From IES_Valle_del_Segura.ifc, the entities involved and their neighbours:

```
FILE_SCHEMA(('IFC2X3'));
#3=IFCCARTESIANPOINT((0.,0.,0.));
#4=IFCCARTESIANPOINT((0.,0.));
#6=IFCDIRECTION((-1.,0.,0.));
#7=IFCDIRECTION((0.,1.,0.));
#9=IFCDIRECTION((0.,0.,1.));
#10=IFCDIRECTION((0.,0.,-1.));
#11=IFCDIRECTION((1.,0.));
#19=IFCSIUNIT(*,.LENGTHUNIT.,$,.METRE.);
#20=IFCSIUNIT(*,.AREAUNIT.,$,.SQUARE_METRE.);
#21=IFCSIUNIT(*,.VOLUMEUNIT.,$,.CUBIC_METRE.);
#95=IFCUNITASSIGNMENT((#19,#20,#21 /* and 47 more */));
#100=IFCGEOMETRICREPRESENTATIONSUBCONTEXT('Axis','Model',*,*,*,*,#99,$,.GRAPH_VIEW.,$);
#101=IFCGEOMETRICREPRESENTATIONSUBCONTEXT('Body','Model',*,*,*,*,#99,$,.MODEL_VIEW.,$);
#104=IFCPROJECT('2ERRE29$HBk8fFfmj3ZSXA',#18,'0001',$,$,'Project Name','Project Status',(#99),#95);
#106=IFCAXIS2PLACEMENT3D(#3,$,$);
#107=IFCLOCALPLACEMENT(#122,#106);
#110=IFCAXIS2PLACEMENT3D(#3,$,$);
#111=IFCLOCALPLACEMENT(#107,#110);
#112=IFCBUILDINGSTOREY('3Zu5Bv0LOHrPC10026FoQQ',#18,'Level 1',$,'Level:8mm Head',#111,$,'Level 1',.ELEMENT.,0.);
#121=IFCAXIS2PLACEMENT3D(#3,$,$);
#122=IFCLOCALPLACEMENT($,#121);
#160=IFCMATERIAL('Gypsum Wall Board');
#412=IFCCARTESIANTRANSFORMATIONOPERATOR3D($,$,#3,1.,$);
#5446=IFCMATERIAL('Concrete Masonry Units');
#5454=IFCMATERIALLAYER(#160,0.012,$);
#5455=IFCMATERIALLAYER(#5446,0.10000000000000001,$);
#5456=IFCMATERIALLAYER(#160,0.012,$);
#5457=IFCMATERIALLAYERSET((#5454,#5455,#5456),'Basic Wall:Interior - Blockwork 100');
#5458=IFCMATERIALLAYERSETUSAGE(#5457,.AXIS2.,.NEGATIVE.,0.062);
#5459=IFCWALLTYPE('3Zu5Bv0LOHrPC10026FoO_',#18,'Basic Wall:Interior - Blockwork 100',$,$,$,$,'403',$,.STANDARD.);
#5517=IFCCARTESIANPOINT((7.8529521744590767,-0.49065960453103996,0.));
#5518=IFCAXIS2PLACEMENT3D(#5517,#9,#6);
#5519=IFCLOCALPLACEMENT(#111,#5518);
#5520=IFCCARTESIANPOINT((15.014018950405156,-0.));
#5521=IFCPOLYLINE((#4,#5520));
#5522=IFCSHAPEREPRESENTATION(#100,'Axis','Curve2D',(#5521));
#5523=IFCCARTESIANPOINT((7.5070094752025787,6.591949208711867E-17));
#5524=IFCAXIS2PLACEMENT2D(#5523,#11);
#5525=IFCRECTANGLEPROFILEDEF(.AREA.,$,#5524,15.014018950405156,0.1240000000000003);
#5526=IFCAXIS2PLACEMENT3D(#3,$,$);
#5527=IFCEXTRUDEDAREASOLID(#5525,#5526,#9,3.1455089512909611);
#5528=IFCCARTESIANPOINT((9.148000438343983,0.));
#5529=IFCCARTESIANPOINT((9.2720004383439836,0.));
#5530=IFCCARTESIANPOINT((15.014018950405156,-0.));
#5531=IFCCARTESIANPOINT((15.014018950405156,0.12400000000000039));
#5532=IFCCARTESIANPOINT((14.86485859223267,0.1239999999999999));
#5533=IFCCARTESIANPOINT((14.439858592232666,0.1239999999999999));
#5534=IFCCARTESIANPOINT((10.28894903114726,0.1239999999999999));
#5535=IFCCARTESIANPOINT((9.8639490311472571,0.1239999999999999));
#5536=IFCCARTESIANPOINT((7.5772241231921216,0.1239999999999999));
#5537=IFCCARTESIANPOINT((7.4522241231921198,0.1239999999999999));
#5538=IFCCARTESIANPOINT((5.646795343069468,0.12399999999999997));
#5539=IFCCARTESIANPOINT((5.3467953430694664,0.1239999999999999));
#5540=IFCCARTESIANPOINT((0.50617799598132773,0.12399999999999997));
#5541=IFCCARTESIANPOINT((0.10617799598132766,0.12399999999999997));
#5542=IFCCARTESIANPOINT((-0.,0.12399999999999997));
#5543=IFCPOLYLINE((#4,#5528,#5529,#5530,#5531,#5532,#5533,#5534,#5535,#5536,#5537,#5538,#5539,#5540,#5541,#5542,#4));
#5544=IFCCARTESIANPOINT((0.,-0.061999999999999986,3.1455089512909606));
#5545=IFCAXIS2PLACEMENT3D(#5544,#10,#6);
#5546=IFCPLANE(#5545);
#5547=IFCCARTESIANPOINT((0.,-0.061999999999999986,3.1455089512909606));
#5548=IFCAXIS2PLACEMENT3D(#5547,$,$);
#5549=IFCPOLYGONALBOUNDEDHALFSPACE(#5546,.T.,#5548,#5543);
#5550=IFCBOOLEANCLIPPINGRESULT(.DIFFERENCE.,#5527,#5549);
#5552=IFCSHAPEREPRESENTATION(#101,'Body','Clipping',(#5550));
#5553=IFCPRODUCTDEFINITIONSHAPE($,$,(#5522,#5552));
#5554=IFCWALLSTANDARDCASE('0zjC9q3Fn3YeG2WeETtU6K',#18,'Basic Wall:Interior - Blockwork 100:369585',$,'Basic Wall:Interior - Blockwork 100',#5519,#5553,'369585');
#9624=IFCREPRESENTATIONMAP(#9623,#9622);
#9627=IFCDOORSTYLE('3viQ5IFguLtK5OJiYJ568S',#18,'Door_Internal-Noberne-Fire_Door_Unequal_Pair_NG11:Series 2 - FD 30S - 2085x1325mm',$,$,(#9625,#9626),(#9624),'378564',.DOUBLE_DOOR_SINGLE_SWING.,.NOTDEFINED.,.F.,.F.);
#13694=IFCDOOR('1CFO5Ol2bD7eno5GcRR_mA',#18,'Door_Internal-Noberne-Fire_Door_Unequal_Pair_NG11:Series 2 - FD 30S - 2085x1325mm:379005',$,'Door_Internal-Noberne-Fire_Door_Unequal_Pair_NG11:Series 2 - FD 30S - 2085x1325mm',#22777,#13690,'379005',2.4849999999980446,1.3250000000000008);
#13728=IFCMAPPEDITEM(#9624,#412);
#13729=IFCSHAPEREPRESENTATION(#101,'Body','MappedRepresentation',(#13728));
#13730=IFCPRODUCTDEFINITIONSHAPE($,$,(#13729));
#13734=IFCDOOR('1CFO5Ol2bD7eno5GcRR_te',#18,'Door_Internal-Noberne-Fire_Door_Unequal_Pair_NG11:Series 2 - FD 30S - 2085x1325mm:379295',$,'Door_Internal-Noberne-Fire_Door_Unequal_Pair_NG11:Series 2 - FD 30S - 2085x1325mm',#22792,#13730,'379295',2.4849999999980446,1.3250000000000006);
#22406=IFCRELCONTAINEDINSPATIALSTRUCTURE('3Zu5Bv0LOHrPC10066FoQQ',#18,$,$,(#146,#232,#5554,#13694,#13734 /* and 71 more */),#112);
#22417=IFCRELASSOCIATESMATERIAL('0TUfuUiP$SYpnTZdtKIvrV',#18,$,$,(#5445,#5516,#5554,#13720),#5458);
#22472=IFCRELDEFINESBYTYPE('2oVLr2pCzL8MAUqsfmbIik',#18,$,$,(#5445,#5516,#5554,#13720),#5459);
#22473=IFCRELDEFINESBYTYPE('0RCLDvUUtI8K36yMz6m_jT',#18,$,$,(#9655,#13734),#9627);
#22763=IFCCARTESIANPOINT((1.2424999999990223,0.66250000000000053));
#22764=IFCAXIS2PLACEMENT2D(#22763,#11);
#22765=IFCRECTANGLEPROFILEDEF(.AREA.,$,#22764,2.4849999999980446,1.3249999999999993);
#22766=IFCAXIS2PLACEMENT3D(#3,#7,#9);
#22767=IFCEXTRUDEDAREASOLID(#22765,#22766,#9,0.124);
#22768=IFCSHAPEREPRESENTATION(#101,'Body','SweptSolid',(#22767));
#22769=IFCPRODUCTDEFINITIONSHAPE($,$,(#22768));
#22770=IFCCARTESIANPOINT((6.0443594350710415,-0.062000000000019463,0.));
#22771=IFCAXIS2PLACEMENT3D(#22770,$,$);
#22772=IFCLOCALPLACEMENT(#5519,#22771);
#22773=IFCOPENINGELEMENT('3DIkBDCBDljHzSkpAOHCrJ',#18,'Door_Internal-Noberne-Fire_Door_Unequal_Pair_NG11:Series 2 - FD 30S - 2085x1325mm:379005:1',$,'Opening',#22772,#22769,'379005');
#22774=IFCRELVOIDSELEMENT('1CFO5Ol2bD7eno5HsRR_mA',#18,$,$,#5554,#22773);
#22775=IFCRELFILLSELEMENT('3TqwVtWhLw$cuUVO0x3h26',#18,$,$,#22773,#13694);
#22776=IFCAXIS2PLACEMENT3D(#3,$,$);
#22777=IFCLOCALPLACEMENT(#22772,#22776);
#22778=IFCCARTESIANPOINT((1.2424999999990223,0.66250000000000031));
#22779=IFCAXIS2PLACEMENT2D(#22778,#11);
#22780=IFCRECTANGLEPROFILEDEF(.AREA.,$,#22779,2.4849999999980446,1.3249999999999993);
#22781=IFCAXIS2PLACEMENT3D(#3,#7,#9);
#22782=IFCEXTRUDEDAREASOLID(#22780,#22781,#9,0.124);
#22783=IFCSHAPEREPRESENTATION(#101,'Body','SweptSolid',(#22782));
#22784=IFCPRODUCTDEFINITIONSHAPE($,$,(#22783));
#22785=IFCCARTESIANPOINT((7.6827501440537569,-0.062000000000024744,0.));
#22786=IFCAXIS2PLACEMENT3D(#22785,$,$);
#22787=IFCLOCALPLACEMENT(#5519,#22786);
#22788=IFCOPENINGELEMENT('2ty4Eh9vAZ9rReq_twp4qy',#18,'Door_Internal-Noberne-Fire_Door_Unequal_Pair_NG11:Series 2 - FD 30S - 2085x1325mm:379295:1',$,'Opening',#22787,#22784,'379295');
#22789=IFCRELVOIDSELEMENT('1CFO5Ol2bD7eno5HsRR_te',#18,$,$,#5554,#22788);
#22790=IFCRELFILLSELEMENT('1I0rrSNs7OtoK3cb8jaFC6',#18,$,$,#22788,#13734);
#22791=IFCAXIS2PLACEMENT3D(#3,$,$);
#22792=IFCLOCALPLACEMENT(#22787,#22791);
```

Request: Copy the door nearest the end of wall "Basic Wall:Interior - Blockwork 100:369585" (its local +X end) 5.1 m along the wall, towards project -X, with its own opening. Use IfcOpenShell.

```python
import ifcopenshell
import ifcopenshell.api.feature
import ifcopenshell.api.geometry
import ifcopenshell.api.root
import ifcopenshell.geom
import ifcopenshell.util.element
import ifcopenshell.util.placement
import ifcopenshell.util.shape
import ifcopenshell.util.unit

model = ifcopenshell.open("IES_Valle_del_Segura.ifc")
unit_scale = ifcopenshell.util.unit.calculate_unit_scale(model)
settings = ifcopenshell.geom.settings()


def volume(element):
    """Net volume in cubic metres, openings subtracted."""
    shape = ifcopenshell.geom.create_shape(settings, element)
    return ifcopenshell.util.shape.get_volume(shape.geometry)


door = model.by_id(13734)
opening = door.FillsVoids[0].RelatingOpeningElement
wall = opening.VoidsElements[0].RelatingBuildingElement
before = volume(wall)
shift = ifcopenshell.util.placement.get_local_placement(wall.ObjectPlacement)[:3, 0] * 5.1 / unit_scale

# copy_class copies the void relationship, type, container and properties, but no geometry.
new_opening = ifcopenshell.api.root.copy_class(model, product=opening)
new_opening.Representation = ifcopenshell.util.element.copy_deep(
    model, opening.Representation, exclude=["IfcGeometricRepresentationContext", "IfcRepresentationMap"]
)
new_opening.Name = "Door_Internal-Noberne-Fire_Door_Unequal_Pair_NG11:Series 2 - FD 30S - 2085x1325mm"
new_opening.Tag = None
new_door = ifcopenshell.api.root.copy_class(model, product=door)
new_door.Representation = ifcopenshell.util.element.copy_deep(
    model, door.Representation, exclude=["IfcGeometricRepresentationContext", "IfcRepresentationMap"]
)
new_door.Name = "Door_Internal-Noberne-Fire_Door_Unequal_Pair_NG11:Series 2 - FD 30S - 2085x1325mm"
new_door.Tag = None
fills = ifcopenshell.api.feature.add_filling(model, opening=new_opening, element=new_door)
fills.OwnerHistory = new_door.OwnerHistory  # required in IFC2X3

for old, new in ((opening, new_opening), (door, new_door)):
    matrix = ifcopenshell.util.placement.get_local_placement(old.ObjectPlacement)
    matrix[:3, 3] += shift
    ifcopenshell.api.geometry.edit_object_placement(model, product=new, matrix=matrix, is_si=False)

after = volume(wall)

print(f"wall volume {before:.3f} -> {after:.3f} m3")

model.write("IES_Valle_del_Segura_v2.ifc")
```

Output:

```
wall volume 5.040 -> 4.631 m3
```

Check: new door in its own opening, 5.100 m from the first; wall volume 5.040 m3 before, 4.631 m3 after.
